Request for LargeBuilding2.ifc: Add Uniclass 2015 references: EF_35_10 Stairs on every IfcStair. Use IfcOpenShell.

First a look at what the model holds.

```python
import ifcopenshell

model = ifcopenshell.open("LargeBuilding2.ifc")
print(model.schema)
print("classifications:", [c.Name for c in model.by_type("IfcClassification")])
for ifc_class in ("IfcDoor", "IfcRoof", "IfcStair", "IfcWall", "IfcWindow"):
    print(ifc_class, len(model.by_type(ifc_class)))
```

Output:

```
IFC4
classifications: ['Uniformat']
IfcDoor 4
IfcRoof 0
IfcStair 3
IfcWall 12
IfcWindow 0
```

```python
import ifcopenshell
import ifcopenshell.api.classification

model = ifcopenshell.open("LargeBuilding2.ifc")

system = ifcopenshell.api.classification.add_classification(model, classification="Uniclass 2015")

codes = {
    "IfcStair": ("EF_35_10", "Stairs"),
}
for ifc_class, (code, name) in codes.items():
    products = model.by_type(ifc_class)
    ifcopenshell.api.classification.add_reference(
        model, products=products, classification=system, identification=code, name=name
    )
    print(code, len(products))

model.write("LargeBuilding2_edited.ifc")
```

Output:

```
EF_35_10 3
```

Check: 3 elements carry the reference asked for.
